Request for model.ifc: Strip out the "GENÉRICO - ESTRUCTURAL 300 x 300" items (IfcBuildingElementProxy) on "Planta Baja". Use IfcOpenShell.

First a look at what the model holds.

```python
import ifcopenshell
import ifcopenshell.util.element

model = ifcopenshell.open("model.ifc")
print(model.schema)
storey = next(s for s in model.by_type("IfcBuildingStorey") if s.Name == "Planta Baja")
proxies = [e for e in ifcopenshell.util.element.get_decomposition(storey) if e.is_a("IfcBuildingElementProxy")]
seen = {}
for e in proxies:
    element_type = ifcopenshell.util.element.get_type(e)
    name = element_type.Name if element_type not in (None, e) else None
    seen[name] = seen.get(name, 0) + 1
for name, count in sorted(seen.items(), key=str):
    print(count, "x", name)
```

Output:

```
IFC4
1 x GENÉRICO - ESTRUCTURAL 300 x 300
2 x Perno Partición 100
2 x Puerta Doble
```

```python
import ifcopenshell
import ifcopenshell.api.root
import ifcopenshell.util.element

model = ifcopenshell.open("model.ifc")

storey = next(s for s in model.by_type("IfcBuildingStorey") if s.Name == "Planta Baja")
proxies = [e for e in ifcopenshell.util.element.get_decomposition(storey) if e.is_a("IfcBuildingElementProxy")]
targets = [e for e in proxies if (t := ifcopenshell.util.element.get_type(e)) not in (None, e) and t.Name == "GENÉRICO - ESTRUCTURAL 300 x 300"]

for e in targets:
    ifcopenshell.api.root.remove_product(model, product=e)
print(len(targets), "removed")

model.write("model-out.ifc")
```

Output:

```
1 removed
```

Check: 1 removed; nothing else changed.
